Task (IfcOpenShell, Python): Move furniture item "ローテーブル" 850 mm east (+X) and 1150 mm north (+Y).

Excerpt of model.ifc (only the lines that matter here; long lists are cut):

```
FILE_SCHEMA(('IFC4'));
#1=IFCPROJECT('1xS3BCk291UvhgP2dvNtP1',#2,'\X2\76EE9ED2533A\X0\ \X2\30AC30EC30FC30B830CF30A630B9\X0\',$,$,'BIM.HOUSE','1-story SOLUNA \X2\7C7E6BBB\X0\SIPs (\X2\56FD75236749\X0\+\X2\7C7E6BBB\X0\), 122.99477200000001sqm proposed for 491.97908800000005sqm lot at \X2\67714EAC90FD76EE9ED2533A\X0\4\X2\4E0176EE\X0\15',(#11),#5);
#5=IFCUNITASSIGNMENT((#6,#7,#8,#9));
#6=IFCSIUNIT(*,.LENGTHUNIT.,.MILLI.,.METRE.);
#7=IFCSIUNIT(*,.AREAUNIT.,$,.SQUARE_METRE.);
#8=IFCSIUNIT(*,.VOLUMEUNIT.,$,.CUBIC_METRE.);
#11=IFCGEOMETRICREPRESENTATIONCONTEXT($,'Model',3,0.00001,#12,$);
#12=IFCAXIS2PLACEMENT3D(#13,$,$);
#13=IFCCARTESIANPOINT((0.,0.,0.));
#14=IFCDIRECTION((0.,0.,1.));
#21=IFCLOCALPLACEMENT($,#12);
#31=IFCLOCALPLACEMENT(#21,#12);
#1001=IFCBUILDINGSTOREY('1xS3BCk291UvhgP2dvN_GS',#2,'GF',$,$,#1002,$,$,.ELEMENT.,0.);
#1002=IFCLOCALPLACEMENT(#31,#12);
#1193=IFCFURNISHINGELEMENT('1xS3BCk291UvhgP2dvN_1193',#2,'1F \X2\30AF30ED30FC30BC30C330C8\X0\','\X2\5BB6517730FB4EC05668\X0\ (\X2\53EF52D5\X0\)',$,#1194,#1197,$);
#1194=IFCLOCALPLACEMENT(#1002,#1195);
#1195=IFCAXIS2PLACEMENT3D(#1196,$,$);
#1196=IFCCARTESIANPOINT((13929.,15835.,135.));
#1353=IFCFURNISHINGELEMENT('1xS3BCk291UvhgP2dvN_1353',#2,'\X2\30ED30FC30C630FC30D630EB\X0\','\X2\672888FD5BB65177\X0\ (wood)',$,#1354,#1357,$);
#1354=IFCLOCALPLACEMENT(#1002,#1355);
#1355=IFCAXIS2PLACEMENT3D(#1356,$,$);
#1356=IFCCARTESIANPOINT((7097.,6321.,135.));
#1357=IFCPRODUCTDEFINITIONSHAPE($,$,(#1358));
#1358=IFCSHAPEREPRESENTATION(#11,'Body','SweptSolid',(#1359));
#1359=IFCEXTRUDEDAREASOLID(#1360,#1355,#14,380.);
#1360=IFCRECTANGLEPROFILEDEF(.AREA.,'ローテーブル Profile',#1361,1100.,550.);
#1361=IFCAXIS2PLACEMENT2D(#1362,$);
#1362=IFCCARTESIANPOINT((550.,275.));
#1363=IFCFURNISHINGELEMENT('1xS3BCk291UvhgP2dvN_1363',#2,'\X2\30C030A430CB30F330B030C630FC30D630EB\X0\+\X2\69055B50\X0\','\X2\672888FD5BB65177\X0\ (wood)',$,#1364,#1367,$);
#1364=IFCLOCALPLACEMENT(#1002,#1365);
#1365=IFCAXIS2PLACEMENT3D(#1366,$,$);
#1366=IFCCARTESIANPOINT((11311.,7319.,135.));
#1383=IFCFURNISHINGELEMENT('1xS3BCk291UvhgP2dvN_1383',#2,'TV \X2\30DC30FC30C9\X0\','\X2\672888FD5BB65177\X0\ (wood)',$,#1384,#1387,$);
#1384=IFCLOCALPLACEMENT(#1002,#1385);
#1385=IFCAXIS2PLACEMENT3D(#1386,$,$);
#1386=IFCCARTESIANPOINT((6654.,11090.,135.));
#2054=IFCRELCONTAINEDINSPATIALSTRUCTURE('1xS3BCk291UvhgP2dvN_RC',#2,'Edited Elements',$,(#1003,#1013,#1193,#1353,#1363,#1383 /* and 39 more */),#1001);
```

```python
import ifcopenshell
import ifcopenshell.api.geometry
import ifcopenshell.util.placement
import ifcopenshell.util.unit

model = ifcopenshell.open("model.ifc")
unit_scale = ifcopenshell.util.unit.calculate_unit_scale(model)

item = model.by_guid("1xS3BCk291UvhgP2dvN_1353")
matrix = ifcopenshell.util.placement.get_local_placement(item.ObjectPlacement)
matrix[0, 3] += 0.85 / unit_scale
matrix[1, 3] += 1.15 / unit_scale
ifcopenshell.api.geometry.edit_object_placement(model, product=item, matrix=matrix, is_si=False)

print(ifcopenshell.util.placement.get_local_placement(item.ObjectPlacement).round(3) + 0.0)

model.write("model_rev.ifc")
```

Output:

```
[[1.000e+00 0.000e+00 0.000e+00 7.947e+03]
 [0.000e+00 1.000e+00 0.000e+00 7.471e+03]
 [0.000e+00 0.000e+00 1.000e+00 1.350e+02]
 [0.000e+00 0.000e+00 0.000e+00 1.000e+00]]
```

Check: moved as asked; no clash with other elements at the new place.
